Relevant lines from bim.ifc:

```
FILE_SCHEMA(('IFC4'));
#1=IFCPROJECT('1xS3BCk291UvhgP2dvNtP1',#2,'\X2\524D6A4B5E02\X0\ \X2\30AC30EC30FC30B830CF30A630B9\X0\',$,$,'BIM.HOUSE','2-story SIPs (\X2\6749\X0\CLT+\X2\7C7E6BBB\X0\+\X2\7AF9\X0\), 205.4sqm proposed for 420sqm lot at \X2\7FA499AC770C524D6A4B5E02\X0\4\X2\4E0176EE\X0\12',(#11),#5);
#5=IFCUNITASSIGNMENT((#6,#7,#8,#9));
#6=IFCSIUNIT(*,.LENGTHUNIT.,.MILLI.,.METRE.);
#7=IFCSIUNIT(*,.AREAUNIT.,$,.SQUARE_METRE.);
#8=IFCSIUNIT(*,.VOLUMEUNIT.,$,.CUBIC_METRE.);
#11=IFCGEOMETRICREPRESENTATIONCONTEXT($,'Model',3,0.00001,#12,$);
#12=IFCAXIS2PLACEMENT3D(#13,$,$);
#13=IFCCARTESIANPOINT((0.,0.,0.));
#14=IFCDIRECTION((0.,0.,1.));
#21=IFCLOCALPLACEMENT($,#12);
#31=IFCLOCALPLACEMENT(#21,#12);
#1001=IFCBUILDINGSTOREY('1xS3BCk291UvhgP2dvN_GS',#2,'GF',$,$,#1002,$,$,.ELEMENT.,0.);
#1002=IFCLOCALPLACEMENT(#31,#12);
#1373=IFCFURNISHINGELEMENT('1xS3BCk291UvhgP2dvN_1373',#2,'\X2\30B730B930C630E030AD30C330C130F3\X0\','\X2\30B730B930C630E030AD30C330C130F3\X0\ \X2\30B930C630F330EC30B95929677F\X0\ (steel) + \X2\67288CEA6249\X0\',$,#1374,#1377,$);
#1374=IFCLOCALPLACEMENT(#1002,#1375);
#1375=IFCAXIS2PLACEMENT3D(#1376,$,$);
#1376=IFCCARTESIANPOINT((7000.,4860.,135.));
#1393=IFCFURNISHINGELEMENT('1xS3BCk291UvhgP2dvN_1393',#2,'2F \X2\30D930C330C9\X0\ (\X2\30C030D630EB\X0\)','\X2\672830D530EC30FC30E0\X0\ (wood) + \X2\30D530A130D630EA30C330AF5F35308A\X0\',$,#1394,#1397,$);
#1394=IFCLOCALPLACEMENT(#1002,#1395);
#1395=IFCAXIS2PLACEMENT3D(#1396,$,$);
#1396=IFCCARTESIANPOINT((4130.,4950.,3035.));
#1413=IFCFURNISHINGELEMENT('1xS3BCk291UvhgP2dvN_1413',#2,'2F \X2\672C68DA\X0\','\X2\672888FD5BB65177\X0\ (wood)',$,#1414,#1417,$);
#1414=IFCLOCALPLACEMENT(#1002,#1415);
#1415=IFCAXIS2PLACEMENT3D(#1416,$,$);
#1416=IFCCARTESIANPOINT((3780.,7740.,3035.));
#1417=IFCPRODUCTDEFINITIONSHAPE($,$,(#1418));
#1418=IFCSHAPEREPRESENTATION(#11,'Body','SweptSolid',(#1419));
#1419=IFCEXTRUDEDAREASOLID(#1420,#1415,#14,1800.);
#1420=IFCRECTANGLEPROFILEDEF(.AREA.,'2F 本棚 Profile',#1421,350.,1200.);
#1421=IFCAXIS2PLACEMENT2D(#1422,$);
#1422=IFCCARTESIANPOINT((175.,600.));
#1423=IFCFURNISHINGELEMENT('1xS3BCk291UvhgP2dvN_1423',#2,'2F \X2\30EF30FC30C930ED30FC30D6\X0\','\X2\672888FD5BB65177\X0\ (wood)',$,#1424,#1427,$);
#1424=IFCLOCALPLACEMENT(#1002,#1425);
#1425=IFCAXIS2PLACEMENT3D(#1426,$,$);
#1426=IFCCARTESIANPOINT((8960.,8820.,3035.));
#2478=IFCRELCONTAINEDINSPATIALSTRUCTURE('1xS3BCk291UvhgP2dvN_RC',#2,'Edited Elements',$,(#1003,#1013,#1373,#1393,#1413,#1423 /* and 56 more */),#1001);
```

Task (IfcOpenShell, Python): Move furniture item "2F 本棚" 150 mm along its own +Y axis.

```python
import ifcopenshell
import ifcopenshell.api.geometry
import ifcopenshell.util.placement
import ifcopenshell.util.unit

model = ifcopenshell.open("bim.ifc")
unit_scale = ifcopenshell.util.unit.calculate_unit_scale(model)

item = model.by_guid("1xS3BCk291UvhgP2dvN_1413")
matrix = ifcopenshell.util.placement.get_local_placement(item.ObjectPlacement)
matrix[:3, 3] += matrix[:3, 1] * 0.15 / unit_scale
ifcopenshell.api.geometry.edit_object_placement(model, product=item, matrix=matrix, is_si=False)

print(ifcopenshell.util.placement.get_local_placement(item.ObjectPlacement).round(3) + 0.0)

model.write("bim_edited.ifc")
```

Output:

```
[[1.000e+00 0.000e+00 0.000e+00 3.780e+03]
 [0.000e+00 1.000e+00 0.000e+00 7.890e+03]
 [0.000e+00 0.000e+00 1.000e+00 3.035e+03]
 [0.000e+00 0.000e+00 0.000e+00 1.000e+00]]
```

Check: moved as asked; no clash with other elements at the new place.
